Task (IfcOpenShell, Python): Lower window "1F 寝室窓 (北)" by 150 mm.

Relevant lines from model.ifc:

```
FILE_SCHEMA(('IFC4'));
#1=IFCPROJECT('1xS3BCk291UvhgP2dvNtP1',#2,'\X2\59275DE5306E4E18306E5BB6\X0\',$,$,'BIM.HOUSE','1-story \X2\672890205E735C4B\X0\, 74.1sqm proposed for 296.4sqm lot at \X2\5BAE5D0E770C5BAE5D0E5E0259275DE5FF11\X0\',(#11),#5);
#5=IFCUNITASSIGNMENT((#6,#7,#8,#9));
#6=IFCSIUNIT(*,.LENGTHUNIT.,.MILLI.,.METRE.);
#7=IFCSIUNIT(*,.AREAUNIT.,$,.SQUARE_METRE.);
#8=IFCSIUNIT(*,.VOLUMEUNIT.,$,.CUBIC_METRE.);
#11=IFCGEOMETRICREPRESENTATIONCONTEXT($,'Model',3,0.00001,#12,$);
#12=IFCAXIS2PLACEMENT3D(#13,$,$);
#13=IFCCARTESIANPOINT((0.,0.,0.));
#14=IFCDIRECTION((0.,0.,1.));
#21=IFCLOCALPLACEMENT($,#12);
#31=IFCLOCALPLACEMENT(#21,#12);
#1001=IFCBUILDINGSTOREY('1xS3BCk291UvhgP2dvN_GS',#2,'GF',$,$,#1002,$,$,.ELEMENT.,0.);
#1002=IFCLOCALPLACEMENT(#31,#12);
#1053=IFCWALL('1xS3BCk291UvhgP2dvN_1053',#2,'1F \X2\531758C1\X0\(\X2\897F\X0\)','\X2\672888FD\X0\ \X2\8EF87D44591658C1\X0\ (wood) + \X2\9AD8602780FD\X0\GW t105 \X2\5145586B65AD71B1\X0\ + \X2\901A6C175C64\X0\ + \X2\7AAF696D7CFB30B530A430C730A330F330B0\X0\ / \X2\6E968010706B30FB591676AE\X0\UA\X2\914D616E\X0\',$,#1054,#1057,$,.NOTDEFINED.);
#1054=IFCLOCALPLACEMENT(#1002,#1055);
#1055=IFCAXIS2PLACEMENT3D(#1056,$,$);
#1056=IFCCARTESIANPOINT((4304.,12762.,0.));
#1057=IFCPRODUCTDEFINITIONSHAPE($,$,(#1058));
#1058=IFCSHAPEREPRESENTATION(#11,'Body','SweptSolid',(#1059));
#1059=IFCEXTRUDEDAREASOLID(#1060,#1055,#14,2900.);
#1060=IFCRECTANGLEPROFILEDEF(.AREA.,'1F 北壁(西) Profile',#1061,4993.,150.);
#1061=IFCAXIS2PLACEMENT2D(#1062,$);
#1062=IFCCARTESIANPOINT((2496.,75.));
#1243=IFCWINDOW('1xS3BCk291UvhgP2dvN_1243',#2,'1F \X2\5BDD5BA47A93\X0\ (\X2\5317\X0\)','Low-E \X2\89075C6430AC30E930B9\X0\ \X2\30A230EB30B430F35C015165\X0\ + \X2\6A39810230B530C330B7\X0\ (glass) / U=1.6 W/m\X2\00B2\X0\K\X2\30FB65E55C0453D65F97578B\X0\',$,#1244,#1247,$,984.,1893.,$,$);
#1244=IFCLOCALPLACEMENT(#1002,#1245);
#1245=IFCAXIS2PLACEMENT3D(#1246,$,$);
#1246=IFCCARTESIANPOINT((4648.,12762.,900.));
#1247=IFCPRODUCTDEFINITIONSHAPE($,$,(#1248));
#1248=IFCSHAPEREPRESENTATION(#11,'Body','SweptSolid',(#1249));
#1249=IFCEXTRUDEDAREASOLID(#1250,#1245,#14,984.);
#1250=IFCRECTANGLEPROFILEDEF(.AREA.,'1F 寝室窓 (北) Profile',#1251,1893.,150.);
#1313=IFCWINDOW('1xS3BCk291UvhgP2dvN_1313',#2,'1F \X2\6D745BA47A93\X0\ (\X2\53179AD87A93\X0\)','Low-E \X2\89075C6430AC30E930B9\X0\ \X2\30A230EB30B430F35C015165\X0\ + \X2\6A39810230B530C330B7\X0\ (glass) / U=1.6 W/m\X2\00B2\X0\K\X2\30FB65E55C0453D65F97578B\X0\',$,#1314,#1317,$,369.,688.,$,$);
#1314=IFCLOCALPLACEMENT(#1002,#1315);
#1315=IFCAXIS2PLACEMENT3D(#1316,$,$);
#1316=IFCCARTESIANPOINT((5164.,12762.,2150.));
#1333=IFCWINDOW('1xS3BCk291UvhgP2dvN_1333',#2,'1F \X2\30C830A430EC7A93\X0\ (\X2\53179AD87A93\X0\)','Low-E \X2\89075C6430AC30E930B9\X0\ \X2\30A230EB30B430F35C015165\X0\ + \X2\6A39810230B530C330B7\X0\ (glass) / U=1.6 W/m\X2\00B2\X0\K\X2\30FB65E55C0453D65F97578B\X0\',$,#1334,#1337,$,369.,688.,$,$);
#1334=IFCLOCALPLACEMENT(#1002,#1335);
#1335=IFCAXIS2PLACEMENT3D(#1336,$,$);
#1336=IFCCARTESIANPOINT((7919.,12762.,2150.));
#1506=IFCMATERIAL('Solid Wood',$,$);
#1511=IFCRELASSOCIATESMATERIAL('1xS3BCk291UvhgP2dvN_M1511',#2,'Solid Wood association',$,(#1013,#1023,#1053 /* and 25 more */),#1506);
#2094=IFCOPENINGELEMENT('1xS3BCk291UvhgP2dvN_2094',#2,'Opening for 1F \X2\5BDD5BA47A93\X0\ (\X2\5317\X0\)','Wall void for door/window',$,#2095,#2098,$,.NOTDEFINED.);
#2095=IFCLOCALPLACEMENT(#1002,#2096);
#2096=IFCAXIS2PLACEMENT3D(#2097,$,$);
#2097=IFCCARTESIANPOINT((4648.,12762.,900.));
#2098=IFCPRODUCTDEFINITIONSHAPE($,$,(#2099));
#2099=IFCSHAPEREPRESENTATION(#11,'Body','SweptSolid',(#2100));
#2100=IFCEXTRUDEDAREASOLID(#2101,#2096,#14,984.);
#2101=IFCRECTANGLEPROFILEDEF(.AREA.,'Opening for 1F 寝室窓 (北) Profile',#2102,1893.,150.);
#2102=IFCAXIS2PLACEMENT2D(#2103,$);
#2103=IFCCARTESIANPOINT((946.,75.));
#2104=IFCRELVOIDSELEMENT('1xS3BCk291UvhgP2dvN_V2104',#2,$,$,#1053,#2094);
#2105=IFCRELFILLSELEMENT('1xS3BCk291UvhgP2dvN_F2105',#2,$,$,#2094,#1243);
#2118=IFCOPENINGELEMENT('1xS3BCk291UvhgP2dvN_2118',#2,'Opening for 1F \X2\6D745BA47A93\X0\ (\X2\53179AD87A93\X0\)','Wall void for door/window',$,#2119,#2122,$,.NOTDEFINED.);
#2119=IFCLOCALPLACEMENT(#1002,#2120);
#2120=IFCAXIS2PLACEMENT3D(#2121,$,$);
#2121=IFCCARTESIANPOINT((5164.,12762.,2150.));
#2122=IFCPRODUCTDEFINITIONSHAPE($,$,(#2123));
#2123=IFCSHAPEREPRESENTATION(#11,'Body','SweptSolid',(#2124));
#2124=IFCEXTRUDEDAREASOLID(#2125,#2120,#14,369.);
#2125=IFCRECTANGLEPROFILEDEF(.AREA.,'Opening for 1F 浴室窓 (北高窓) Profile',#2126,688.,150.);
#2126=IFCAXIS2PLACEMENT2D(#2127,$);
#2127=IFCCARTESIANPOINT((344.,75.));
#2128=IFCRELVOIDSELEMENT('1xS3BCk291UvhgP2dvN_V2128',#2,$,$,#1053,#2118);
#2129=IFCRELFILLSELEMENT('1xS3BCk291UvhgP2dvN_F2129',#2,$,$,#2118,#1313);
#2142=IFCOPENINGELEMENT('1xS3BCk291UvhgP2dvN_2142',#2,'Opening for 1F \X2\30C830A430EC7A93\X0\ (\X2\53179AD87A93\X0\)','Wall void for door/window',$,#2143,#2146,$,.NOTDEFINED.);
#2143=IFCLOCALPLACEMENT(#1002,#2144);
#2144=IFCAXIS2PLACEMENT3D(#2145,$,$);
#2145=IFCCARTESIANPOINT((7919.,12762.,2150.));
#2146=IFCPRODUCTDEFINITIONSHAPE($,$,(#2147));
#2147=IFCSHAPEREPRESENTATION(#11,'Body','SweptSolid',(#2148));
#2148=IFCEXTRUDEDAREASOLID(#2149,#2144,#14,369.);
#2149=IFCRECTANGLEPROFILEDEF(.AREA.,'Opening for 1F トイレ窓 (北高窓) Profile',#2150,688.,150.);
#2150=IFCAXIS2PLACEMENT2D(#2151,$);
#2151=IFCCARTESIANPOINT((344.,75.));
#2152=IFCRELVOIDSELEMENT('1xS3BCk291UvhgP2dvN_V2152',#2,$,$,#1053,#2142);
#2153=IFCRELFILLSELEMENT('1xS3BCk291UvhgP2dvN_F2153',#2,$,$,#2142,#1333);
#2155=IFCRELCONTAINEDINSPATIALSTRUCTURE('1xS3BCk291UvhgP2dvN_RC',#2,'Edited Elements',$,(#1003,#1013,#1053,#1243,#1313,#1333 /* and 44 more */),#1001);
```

```python
import numpy as np
import ifcopenshell
import ifcopenshell.api.geometry
import ifcopenshell.util.placement
import ifcopenshell.util.unit

model = ifcopenshell.open("model.ifc")
unit_scale = ifcopenshell.util.unit.calculate_unit_scale(model)

window = model.by_guid("1xS3BCk291UvhgP2dvN_1243")
opening = window.FillsVoids[0].RelatingOpeningElement
dz = -150.0

shift = np.array([0.0, 0.0, dz])
# The window is not placed relative to its opening, so move both.
for product in (opening, window):
    matrix = ifcopenshell.util.placement.get_local_placement(product.ObjectPlacement)
    matrix[:3, 3] += shift
    ifcopenshell.api.geometry.edit_object_placement(model, product=product, matrix=matrix, is_si=False)

print(f"moved by {dz * unit_scale:+.3f} m")

model.write("model_rev.ifc")
```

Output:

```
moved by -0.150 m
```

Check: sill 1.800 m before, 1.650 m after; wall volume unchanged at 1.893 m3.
